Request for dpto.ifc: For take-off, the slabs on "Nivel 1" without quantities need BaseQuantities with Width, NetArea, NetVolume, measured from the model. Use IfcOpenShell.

First a look at what the model holds.

```python
import ifcopenshell
import ifcopenshell.util.element
import ifcopenshell.util.unit

model = ifcopenshell.open("dpto.ifc")
print(model.schema)
for unit_type in ("LENGTHUNIT", "AREAUNIT", "VOLUMEUNIT"):
    print(unit_type, ifcopenshell.util.unit.calculate_unit_scale(model, unit_type))
storey = next(s for s in model.by_type("IfcBuildingStorey") if s.Name == "Nivel 1")
slabs = [e for e in ifcopenshell.util.element.get_decomposition(storey) if e.is_a("IfcSlab")]
for e in sorted(slabs, key=lambda e: e.id()):
    print(e.id(), e.is_a(), e.Name, list(ifcopenshell.util.element.get_psets(e, qtos_only=True)), sep=" | ")
```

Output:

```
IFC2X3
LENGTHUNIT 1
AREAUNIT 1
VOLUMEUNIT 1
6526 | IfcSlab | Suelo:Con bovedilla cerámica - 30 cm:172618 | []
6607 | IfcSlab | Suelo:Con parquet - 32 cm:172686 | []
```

```python
import ifcopenshell
import ifcopenshell.api.pset
import ifcopenshell.geom
import ifcopenshell.util.element
import ifcopenshell.util.shape
import ifcopenshell.util.unit

model = ifcopenshell.open("dpto.ifc")
unit_scale = ifcopenshell.util.unit.calculate_unit_scale(model)
area_scale = ifcopenshell.util.unit.calculate_unit_scale(model, "AREAUNIT")
volume_scale = ifcopenshell.util.unit.calculate_unit_scale(model, "VOLUMEUNIT")
settings = ifcopenshell.geom.settings()

storey = next(s for s in model.by_type("IfcBuildingStorey") if s.Name == "Nivel 1")
slabs = [e for e in ifcopenshell.util.element.get_decomposition(storey) if e.is_a("IfcSlab")]

for e in sorted(slabs, key=lambda e: e.id()):
    if ifcopenshell.util.element.get_psets(e, qtos_only=True, should_inherit=False):
        continue
    # Geometry comes back in metres, in the element's own axes.
    shape = ifcopenshell.geom.create_shape(settings, e)
    values = {
        "Width": ifcopenshell.util.shape.get_z(shape.geometry) / unit_scale,
        "NetArea": ifcopenshell.util.shape.get_footprint_area(shape.geometry) / area_scale,
        "NetVolume": ifcopenshell.util.shape.get_volume(shape.geometry) / volume_scale,
    }
    qto = ifcopenshell.api.pset.add_qto(model, product=e, name="BaseQuantities")
    ifcopenshell.api.pset.edit_qto(model, qto=qto, properties=values)
    print(e.id(), {k: round(v, 3) for k, v in values.items()})

model.write("dpto_updated.ifc")
```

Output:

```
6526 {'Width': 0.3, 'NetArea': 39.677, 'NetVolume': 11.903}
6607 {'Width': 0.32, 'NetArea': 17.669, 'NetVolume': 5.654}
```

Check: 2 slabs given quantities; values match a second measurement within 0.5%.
